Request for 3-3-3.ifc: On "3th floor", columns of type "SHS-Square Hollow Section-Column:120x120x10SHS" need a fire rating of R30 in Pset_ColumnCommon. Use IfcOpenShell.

First a look at what the model holds.

```python
import ifcopenshell
import ifcopenshell.util.element

model = ifcopenshell.open("3-3-3.ifc")
print(model.schema)
storey = next(s for s in model.by_type("IfcBuildingStorey") if s.Name == "3th floor")
columns = [e for e in ifcopenshell.util.element.get_decomposition(storey) if e.is_a("IfcColumn")]
seen = {}
for e in columns:
    element_type = ifcopenshell.util.element.get_type(e)
    key = (element_type.Name if element_type != e and element_type else None, ifcopenshell.util.element.get_pset(e, "Pset_ColumnCommon", "FireRating"))
    seen[key] = seen.get(key, 0) + 1
for (name, value), count in sorted(seen.items(), key=str):
    print(count, "x", name, "|", value)
```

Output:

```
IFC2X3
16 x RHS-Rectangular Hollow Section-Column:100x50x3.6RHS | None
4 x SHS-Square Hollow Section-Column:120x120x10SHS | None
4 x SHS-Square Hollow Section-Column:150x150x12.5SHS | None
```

```python
import ifcopenshell
import ifcopenshell.api.pset
import ifcopenshell.util.element

model = ifcopenshell.open("3-3-3.ifc")

storey = next(s for s in model.by_type("IfcBuildingStorey") if s.Name == "3th floor")
columns = [e for e in ifcopenshell.util.element.get_decomposition(storey) if e.is_a("IfcColumn")]

count = 0
for e in columns:
    element_type = ifcopenshell.util.element.get_type(e)
    if element_type in (None, e) or element_type.Name != "SHS-Square Hollow Section-Column:120x120x10SHS":
        continue
    # add_pset returns the element's existing set when there is one.
    pset = ifcopenshell.api.pset.add_pset(model, product=e, name="Pset_ColumnCommon")
    ifcopenshell.api.pset.edit_pset(model, pset=pset, properties={"FireRating": "R30"})
    count += 1

print(count, "columns updated")

model.write("3-3-3-out.ifc")
```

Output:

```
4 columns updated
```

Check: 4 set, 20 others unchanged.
